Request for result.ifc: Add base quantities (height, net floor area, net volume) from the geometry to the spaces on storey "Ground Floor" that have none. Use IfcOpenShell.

First a look at what the model holds.

```python
import ifcopenshell
import ifcopenshell.util.element
import ifcopenshell.util.unit

model = ifcopenshell.open("result.ifc")
print(model.schema)
for unit_type in ("LENGTHUNIT", "AREAUNIT", "VOLUMEUNIT"):
    print(unit_type, ifcopenshell.util.unit.calculate_unit_scale(model, unit_type))
storey = next(s for s in model.by_type("IfcBuildingStorey") if s.Name == "Ground Floor")
spaces = [e for e in ifcopenshell.util.element.get_decomposition(storey) if e.is_a("IfcSpace")]
for e in sorted(spaces, key=lambda e: e.id()):
    print(e.id(), e.is_a(), e.Name, list(ifcopenshell.util.element.get_psets(e, qtos_only=True)), sep=" | ")
```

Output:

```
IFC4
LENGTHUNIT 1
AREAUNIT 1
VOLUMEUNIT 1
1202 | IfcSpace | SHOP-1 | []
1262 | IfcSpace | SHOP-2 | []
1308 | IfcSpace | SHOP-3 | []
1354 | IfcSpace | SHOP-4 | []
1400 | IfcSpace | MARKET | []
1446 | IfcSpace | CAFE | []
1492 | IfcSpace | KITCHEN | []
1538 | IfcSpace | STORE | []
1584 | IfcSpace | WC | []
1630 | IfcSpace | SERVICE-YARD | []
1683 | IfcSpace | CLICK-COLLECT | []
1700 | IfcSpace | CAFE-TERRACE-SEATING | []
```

```python
import ifcopenshell
import ifcopenshell.api.pset
import ifcopenshell.geom
import ifcopenshell.util.element
import ifcopenshell.util.shape
import ifcopenshell.util.unit

model = ifcopenshell.open("result.ifc")
unit_scale = ifcopenshell.util.unit.calculate_unit_scale(model)
area_scale = ifcopenshell.util.unit.calculate_unit_scale(model, "AREAUNIT")
volume_scale = ifcopenshell.util.unit.calculate_unit_scale(model, "VOLUMEUNIT")
settings = ifcopenshell.geom.settings()

storey = next(s for s in model.by_type("IfcBuildingStorey") if s.Name == "Ground Floor")
spaces = [e for e in ifcopenshell.util.element.get_decomposition(storey) if e.is_a("IfcSpace")]

for e in sorted(spaces, key=lambda e: e.id()):
    if ifcopenshell.util.element.get_psets(e, qtos_only=True, should_inherit=False):
        continue
    # Geometry comes back in metres, in the element's own axes.
    shape = ifcopenshell.geom.create_shape(settings, e)
    values = {
        "Height": ifcopenshell.util.shape.get_z(shape.geometry) / unit_scale,
        "NetFloorArea": ifcopenshell.util.shape.get_footprint_area(shape.geometry) / area_scale,
        "NetVolume": ifcopenshell.util.shape.get_volume(shape.geometry) / volume_scale,
    }
    qto = ifcopenshell.api.pset.add_qto(model, product=e, name="Qto_SpaceBaseQuantities")
    ifcopenshell.api.pset.edit_qto(model, qto=qto, properties=values)
    print(e.id(), {k: round(v, 3) for k, v in values.items()})

model.write("result-out.ifc")
```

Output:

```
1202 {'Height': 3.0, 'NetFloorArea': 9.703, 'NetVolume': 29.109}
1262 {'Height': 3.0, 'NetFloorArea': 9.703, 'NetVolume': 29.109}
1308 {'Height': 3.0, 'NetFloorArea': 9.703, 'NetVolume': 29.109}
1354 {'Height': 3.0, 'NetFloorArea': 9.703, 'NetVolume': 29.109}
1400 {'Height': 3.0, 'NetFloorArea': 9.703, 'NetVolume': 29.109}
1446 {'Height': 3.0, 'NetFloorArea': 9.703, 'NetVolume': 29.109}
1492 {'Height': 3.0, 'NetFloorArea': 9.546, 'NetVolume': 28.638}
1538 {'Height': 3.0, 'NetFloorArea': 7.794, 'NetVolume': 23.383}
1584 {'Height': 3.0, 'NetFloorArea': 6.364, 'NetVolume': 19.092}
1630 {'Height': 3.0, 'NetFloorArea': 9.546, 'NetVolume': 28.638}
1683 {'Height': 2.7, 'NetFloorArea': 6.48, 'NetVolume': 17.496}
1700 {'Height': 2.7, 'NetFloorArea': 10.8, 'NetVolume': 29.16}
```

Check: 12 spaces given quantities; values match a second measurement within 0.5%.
